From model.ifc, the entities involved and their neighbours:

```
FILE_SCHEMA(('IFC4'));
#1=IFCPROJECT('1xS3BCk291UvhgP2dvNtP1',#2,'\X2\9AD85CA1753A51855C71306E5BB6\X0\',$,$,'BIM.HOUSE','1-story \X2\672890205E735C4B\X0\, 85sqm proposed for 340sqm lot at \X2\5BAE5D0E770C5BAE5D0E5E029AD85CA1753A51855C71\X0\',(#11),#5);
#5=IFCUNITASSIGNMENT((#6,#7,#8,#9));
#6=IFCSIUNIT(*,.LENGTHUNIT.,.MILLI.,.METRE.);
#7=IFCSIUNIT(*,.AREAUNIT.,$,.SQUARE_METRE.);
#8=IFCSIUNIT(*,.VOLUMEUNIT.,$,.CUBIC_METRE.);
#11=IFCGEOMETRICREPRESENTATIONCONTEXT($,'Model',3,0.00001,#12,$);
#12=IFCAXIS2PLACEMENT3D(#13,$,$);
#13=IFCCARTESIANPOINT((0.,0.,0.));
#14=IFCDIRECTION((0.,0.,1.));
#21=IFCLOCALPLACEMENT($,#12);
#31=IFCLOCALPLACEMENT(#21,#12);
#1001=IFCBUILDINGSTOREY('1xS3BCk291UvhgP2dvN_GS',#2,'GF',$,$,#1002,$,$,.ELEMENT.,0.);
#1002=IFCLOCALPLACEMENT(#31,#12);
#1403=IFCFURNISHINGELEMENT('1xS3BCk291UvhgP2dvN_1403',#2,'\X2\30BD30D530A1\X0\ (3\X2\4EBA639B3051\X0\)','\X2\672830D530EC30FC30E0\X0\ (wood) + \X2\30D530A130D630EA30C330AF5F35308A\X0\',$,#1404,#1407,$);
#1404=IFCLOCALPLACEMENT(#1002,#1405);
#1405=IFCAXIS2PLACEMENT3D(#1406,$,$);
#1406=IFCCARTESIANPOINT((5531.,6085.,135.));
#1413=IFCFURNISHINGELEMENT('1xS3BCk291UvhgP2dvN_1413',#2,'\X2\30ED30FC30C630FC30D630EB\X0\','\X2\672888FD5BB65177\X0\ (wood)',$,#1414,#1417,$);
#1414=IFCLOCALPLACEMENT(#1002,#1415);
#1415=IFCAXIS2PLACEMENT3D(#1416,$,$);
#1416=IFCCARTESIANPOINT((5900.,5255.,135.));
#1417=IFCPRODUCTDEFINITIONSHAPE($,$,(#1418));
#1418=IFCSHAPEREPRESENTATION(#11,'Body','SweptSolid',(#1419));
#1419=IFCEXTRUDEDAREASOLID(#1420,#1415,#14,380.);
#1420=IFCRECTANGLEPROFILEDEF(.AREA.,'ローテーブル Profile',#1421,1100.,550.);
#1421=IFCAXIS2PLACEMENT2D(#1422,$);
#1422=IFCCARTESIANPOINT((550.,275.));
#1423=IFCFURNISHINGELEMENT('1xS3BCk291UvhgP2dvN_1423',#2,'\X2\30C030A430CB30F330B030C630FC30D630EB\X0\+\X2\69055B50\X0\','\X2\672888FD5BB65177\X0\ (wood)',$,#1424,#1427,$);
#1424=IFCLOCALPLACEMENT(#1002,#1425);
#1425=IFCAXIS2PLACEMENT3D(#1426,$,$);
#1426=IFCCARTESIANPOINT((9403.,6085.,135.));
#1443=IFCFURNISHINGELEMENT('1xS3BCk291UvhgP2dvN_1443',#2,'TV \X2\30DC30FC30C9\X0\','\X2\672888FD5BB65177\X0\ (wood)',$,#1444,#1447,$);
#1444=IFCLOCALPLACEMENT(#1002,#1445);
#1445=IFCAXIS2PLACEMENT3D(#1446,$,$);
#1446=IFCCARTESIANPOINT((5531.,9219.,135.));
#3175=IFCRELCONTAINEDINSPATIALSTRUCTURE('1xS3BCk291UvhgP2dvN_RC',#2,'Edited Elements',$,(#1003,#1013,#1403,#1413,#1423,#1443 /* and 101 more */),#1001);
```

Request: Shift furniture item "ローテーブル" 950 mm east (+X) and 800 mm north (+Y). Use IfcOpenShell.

```python
import ifcopenshell
import ifcopenshell.api.geometry
import ifcopenshell.util.placement

model = ifcopenshell.open("model.ifc")

item = model.by_id(1413)
matrix = ifcopenshell.util.placement.get_local_placement(item.ObjectPlacement)
matrix[0, 3] += 950.0
matrix[1, 3] += 800.0
ifcopenshell.api.geometry.edit_object_placement(model, product=item, matrix=matrix, is_si=False)

print(ifcopenshell.util.placement.get_local_placement(item.ObjectPlacement).round(3) + 0.0)

model.write("model-out.ifc")
```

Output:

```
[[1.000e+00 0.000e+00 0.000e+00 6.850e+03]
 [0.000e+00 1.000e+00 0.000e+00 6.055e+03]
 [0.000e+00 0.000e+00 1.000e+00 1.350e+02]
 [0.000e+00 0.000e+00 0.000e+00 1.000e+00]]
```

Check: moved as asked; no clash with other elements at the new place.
